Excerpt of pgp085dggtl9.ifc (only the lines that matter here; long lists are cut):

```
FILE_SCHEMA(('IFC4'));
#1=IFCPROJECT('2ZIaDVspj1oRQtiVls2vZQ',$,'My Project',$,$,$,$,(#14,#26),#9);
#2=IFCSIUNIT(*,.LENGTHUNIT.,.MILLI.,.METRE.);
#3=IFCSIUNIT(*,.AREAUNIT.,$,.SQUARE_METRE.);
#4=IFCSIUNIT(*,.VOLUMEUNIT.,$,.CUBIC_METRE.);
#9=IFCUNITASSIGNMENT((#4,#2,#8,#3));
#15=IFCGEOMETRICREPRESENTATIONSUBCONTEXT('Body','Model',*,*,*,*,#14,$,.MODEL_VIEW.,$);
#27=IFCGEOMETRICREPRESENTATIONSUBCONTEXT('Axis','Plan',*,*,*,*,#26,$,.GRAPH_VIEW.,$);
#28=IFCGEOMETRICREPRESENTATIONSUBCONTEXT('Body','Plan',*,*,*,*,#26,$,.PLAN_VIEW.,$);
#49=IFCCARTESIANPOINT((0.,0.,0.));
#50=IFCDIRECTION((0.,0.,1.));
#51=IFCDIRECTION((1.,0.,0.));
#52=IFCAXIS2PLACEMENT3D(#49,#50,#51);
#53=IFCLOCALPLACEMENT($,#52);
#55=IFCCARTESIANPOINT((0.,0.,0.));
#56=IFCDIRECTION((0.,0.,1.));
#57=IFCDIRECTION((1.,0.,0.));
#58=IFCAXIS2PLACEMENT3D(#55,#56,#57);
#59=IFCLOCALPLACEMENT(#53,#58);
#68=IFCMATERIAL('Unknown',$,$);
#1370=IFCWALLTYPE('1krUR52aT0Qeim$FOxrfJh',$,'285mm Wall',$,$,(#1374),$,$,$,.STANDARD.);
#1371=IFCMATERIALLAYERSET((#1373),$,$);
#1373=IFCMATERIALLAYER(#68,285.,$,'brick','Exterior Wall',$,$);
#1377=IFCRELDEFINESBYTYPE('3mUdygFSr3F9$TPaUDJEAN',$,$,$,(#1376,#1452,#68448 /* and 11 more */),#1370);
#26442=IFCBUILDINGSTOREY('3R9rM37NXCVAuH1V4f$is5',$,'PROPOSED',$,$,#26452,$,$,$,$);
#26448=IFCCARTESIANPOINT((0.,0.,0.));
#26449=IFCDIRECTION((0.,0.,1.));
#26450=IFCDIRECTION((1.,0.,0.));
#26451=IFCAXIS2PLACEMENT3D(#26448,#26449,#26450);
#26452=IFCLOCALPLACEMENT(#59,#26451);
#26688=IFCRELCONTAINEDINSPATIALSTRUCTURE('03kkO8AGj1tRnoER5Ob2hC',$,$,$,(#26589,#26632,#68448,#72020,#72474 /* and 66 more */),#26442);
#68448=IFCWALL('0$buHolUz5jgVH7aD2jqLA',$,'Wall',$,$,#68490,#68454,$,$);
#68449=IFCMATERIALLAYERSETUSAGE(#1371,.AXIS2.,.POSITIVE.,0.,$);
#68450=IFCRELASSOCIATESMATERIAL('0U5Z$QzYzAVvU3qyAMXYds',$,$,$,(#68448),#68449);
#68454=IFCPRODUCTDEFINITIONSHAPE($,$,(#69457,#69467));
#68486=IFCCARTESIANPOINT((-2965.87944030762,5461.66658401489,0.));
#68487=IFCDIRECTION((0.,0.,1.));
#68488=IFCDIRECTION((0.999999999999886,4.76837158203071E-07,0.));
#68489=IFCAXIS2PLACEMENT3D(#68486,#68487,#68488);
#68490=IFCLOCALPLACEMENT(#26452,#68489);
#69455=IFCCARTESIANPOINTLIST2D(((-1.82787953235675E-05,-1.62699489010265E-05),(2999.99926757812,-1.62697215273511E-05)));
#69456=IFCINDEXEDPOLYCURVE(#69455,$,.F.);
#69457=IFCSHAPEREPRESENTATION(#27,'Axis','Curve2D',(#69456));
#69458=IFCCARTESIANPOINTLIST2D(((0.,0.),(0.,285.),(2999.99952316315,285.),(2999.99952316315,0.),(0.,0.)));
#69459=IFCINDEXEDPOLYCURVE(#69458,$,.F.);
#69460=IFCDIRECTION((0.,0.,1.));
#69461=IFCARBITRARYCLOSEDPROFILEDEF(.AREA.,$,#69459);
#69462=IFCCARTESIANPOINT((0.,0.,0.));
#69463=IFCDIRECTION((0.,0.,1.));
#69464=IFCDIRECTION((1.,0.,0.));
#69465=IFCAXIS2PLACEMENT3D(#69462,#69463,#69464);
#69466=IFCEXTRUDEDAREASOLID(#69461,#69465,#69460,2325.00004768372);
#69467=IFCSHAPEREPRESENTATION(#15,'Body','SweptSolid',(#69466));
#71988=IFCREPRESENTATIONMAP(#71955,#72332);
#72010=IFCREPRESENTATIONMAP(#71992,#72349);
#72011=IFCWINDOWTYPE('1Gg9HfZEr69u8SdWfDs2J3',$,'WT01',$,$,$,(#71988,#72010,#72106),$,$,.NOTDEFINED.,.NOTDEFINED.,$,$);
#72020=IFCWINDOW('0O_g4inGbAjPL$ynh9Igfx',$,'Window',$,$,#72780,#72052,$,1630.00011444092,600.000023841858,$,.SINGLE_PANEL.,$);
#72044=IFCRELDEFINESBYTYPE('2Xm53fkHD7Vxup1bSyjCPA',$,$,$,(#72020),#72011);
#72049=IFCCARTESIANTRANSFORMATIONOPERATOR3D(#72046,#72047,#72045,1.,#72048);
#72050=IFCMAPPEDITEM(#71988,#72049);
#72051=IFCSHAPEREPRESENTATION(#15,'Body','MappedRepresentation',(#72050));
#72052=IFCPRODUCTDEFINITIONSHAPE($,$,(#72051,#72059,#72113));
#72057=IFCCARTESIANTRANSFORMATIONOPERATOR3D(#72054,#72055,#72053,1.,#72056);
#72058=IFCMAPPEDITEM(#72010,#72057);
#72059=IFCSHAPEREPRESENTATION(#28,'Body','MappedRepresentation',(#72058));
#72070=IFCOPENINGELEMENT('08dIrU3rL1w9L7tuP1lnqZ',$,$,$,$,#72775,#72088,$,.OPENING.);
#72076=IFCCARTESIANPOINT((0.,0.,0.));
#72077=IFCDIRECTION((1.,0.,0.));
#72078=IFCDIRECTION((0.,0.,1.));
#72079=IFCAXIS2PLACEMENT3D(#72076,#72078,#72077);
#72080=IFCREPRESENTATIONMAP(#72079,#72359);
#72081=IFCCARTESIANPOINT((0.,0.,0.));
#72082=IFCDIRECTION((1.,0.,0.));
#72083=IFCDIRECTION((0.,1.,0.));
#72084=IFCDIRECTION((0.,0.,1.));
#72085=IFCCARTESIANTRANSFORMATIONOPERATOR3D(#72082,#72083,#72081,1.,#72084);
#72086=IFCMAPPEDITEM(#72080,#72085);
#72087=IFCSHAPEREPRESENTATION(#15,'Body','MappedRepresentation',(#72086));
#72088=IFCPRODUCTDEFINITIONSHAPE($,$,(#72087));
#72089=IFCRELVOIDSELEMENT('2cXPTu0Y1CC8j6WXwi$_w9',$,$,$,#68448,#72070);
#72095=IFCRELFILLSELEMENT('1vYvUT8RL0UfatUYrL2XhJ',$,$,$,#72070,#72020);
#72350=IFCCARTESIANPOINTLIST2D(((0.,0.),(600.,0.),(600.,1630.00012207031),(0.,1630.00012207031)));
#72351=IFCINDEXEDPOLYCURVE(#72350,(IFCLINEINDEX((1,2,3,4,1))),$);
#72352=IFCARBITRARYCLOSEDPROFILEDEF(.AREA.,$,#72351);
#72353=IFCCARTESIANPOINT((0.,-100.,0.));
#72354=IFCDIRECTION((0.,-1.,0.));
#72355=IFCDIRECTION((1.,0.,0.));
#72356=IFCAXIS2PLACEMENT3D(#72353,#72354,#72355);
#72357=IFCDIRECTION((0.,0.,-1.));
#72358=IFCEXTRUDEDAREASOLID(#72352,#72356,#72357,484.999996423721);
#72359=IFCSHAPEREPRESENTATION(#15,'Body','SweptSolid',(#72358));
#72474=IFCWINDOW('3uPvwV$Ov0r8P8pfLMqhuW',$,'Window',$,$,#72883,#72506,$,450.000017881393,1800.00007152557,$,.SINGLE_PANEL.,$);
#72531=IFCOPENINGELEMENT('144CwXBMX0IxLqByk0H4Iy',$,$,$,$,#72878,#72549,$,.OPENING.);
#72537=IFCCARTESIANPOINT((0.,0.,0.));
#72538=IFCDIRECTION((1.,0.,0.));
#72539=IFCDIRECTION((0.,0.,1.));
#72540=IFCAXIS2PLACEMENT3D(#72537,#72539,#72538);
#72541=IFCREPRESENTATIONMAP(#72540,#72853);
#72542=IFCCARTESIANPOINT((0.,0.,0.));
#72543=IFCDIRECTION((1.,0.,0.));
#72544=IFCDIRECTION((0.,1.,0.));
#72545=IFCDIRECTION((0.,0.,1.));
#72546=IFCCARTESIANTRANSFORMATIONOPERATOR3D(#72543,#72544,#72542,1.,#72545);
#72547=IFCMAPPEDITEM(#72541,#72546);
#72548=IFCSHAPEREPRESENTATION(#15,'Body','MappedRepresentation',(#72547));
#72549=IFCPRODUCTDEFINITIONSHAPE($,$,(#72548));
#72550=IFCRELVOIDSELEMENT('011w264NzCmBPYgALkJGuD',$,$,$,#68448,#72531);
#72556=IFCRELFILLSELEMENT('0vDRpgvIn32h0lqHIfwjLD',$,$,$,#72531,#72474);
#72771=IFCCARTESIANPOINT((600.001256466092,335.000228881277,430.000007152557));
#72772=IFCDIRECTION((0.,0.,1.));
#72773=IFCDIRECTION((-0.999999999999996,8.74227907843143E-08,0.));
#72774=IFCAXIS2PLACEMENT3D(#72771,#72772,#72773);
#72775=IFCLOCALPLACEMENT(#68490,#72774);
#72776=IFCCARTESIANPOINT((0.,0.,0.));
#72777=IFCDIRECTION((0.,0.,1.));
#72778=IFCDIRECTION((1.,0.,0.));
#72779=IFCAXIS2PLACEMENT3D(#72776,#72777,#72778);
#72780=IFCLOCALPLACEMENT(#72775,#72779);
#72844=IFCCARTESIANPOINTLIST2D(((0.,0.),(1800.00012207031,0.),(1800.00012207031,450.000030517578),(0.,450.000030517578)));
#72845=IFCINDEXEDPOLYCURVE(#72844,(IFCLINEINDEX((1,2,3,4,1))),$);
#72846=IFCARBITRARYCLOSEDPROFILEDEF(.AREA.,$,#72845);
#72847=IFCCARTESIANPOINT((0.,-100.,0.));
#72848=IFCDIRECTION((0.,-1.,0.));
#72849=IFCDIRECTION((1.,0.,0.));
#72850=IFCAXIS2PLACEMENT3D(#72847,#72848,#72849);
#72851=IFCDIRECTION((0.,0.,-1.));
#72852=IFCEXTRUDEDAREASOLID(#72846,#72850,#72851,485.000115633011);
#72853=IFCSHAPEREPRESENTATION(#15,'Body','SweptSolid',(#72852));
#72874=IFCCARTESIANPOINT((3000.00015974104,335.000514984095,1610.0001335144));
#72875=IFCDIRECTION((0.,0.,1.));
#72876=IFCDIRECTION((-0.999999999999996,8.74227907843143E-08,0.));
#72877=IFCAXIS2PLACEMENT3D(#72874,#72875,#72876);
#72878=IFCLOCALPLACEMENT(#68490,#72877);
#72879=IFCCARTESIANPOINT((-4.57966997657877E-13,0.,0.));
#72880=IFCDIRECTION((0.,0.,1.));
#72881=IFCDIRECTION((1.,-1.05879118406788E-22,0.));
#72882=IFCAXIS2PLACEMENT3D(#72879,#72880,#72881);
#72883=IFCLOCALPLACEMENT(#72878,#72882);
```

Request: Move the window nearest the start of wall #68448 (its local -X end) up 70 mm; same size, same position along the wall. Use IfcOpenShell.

```python
import numpy as np
import ifcopenshell
import ifcopenshell.api.geometry
import ifcopenshell.util.placement
import ifcopenshell.util.unit

model = ifcopenshell.open("pgp085dggtl9.ifc")
unit_scale = ifcopenshell.util.unit.calculate_unit_scale(model)

window = model.by_guid("0O_g4inGbAjPL$ynh9Igfx")
opening = window.FillsVoids[0].RelatingOpeningElement
dz = 70.0

shift = np.array([0.0, 0.0, dz])
# The window is placed relative to its opening, so it follows when the opening moves.
matrix = ifcopenshell.util.placement.get_local_placement(opening.ObjectPlacement)
matrix[:3, 3] += shift
ifcopenshell.api.geometry.edit_object_placement(
    model, product=opening, matrix=matrix, is_si=False, should_transform_children=True
)

print(f"moved by {dz * unit_scale:+.3f} m")

model.write("pgp085dggtl9_v2.ifc")
```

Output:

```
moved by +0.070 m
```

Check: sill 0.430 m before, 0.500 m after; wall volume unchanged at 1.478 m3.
